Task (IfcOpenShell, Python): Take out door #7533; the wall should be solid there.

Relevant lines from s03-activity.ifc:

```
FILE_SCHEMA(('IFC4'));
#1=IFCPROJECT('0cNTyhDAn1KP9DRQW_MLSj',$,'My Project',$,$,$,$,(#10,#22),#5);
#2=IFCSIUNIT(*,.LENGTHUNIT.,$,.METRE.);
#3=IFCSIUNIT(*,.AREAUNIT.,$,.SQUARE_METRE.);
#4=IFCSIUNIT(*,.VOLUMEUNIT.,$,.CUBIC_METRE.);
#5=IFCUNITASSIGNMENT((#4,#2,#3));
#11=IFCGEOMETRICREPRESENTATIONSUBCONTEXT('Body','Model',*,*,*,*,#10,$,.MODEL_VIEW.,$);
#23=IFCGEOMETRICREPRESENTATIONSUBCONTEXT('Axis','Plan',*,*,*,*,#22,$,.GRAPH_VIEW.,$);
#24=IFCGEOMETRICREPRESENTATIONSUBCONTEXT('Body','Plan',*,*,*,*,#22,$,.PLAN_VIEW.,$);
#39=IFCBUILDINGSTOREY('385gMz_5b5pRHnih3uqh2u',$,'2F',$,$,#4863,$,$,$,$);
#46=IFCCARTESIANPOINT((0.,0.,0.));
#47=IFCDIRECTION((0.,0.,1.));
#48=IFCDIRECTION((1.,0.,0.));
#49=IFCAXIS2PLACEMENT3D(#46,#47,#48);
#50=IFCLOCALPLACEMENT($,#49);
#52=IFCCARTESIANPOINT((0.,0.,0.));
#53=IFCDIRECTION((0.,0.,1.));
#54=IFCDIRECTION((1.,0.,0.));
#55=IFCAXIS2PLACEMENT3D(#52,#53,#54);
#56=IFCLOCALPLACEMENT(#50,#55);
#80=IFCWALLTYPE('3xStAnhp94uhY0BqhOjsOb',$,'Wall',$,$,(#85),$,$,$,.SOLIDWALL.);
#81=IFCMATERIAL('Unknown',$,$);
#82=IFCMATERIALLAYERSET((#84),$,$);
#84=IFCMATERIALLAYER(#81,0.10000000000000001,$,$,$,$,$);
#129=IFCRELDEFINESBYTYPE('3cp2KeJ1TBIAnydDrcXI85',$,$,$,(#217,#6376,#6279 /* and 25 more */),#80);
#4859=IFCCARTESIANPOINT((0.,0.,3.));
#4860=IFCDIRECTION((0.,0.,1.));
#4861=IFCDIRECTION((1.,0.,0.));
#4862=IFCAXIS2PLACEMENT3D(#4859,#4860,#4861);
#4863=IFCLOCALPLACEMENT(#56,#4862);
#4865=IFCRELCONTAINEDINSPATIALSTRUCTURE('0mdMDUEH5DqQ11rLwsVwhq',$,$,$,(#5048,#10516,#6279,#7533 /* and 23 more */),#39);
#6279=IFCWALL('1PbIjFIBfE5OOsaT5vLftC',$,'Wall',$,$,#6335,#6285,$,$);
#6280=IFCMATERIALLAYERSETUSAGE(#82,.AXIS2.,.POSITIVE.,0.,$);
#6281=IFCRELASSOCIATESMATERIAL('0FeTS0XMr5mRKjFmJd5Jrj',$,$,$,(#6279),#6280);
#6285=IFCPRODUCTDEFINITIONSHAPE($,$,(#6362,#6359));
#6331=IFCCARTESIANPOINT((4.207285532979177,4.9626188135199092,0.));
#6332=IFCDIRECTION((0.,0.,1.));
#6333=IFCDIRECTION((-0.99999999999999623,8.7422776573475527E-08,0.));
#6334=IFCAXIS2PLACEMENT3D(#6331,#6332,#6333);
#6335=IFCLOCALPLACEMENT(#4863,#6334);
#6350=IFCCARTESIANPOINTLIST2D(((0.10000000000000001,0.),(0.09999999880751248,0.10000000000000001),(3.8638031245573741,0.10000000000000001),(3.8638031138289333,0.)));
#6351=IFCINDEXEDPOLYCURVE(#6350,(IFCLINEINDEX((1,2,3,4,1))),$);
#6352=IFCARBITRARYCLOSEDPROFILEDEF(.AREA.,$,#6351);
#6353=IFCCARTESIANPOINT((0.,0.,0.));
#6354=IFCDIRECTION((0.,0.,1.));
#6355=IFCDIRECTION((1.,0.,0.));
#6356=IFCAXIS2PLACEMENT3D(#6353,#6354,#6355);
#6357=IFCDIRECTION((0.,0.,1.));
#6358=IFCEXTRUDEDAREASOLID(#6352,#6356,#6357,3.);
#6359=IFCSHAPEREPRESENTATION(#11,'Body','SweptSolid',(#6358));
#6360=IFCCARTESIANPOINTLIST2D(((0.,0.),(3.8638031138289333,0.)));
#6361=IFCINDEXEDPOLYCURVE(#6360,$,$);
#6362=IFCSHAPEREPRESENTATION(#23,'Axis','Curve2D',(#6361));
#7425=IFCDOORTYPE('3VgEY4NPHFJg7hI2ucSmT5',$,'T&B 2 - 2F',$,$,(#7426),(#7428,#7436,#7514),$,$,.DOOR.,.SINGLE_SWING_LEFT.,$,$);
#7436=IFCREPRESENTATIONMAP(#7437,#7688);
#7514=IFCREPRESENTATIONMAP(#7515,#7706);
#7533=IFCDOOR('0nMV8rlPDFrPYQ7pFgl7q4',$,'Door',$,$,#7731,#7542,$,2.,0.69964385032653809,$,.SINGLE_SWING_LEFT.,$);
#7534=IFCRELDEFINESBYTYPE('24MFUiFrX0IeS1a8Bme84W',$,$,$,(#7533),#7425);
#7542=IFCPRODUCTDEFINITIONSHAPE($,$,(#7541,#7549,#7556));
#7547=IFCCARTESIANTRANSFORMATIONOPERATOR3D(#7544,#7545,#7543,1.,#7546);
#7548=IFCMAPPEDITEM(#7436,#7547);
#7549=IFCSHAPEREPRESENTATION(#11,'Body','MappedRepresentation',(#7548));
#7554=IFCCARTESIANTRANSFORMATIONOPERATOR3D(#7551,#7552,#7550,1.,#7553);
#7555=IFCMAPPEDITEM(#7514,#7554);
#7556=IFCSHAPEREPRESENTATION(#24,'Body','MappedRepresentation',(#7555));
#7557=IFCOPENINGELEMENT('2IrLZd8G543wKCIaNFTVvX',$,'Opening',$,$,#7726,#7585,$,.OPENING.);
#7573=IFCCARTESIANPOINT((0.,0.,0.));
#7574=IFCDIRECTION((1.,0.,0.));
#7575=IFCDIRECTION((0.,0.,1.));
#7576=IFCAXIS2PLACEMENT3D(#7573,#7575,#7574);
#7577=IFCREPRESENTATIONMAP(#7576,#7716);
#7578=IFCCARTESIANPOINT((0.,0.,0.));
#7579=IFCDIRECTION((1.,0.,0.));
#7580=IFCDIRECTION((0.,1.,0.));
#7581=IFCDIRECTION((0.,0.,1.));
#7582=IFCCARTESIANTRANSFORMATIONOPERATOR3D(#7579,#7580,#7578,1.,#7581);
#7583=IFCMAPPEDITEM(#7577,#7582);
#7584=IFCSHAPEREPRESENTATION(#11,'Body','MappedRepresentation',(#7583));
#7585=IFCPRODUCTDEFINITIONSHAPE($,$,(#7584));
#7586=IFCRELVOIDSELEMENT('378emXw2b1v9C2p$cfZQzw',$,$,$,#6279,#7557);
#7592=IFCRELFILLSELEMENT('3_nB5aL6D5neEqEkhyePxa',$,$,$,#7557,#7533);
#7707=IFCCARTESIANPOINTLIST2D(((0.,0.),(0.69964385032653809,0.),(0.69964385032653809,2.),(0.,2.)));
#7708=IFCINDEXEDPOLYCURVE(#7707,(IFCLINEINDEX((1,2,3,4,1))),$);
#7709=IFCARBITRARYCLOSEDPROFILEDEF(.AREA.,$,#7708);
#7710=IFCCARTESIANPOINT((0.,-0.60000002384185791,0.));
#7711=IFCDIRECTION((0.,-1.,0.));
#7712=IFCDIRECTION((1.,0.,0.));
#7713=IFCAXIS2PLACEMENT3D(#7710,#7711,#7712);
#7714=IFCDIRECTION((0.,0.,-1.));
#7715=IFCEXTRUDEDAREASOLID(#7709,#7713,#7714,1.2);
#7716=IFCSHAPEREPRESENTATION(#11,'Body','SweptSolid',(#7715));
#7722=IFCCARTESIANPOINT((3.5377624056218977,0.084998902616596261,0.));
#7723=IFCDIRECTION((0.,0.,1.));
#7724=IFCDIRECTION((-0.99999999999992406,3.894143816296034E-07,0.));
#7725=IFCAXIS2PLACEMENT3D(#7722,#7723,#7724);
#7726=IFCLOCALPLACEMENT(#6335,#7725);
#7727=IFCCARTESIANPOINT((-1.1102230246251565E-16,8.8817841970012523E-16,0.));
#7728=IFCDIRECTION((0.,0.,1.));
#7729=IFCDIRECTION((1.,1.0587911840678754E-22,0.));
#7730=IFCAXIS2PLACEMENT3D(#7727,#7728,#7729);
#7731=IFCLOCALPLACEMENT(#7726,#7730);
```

```python
import ifcopenshell
import ifcopenshell.api.feature
import ifcopenshell.api.root
import ifcopenshell.geom
import ifcopenshell.util.shape

model = ifcopenshell.open("s03-activity.ifc")
settings = ifcopenshell.geom.settings()


def volume(element):
    """Net volume in cubic metres, openings subtracted."""
    shape = ifcopenshell.geom.create_shape(settings, element)
    return ifcopenshell.util.shape.get_volume(shape.geometry)


door = model.by_guid("0nMV8rlPDFrPYQ7pFgl7q4")
opening = door.FillsVoids[0].RelatingOpeningElement
wall = opening.VoidsElements[0].RelatingBuildingElement
before = volume(wall)

ifcopenshell.api.root.remove_product(model, product=door)
ifcopenshell.api.feature.remove_feature(model, feature=opening)

after = volume(wall)

print(f"wall volume {before:.3f} -> {after:.3f} m3")

model.write("s03-activity_rev.ifc")
```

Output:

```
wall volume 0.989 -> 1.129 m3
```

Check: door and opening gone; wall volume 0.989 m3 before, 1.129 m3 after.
